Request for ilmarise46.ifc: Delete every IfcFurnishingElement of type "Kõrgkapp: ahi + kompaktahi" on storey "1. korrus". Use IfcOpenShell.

First a look at what the model holds.

```python
import ifcopenshell
import ifcopenshell.util.element

model = ifcopenshell.open("ilmarise46.ifc")
print(model.schema)
storey = next(s for s in model.by_type("IfcBuildingStorey") if s.Name == "1. korrus")
furniture = [e for e in ifcopenshell.util.element.get_decomposition(storey) if e.is_a("IfcFurnishingElement")]
seen = {}
for e in furniture:
    element_type = ifcopenshell.util.element.get_type(e)
    name = element_type.Name if element_type not in (None, e) else None
    seen[name] = seen.get(name, 0) + 1
for name, count in sorted(seen.items(), key=str):
    print(count, "x", name)
```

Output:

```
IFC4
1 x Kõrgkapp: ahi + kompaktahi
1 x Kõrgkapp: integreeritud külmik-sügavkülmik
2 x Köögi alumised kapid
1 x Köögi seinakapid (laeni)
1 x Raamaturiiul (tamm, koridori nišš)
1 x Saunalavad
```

```python
import ifcopenshell
import ifcopenshell.api.root
import ifcopenshell.util.element

model = ifcopenshell.open("ilmarise46.ifc")

storey = next(s for s in model.by_type("IfcBuildingStorey") if s.Name == "1. korrus")
furniture = [e for e in ifcopenshell.util.element.get_decomposition(storey) if e.is_a("IfcFurnishingElement")]
targets = [e for e in furniture if (t := ifcopenshell.util.element.get_type(e)) not in (None, e) and t.Name == "Kõrgkapp: ahi + kompaktahi"]

for e in targets:
    ifcopenshell.api.root.remove_product(model, product=e)
print(len(targets), "removed")

model.write("ilmarise46-out.ifc")
```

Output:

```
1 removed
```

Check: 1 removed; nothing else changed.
